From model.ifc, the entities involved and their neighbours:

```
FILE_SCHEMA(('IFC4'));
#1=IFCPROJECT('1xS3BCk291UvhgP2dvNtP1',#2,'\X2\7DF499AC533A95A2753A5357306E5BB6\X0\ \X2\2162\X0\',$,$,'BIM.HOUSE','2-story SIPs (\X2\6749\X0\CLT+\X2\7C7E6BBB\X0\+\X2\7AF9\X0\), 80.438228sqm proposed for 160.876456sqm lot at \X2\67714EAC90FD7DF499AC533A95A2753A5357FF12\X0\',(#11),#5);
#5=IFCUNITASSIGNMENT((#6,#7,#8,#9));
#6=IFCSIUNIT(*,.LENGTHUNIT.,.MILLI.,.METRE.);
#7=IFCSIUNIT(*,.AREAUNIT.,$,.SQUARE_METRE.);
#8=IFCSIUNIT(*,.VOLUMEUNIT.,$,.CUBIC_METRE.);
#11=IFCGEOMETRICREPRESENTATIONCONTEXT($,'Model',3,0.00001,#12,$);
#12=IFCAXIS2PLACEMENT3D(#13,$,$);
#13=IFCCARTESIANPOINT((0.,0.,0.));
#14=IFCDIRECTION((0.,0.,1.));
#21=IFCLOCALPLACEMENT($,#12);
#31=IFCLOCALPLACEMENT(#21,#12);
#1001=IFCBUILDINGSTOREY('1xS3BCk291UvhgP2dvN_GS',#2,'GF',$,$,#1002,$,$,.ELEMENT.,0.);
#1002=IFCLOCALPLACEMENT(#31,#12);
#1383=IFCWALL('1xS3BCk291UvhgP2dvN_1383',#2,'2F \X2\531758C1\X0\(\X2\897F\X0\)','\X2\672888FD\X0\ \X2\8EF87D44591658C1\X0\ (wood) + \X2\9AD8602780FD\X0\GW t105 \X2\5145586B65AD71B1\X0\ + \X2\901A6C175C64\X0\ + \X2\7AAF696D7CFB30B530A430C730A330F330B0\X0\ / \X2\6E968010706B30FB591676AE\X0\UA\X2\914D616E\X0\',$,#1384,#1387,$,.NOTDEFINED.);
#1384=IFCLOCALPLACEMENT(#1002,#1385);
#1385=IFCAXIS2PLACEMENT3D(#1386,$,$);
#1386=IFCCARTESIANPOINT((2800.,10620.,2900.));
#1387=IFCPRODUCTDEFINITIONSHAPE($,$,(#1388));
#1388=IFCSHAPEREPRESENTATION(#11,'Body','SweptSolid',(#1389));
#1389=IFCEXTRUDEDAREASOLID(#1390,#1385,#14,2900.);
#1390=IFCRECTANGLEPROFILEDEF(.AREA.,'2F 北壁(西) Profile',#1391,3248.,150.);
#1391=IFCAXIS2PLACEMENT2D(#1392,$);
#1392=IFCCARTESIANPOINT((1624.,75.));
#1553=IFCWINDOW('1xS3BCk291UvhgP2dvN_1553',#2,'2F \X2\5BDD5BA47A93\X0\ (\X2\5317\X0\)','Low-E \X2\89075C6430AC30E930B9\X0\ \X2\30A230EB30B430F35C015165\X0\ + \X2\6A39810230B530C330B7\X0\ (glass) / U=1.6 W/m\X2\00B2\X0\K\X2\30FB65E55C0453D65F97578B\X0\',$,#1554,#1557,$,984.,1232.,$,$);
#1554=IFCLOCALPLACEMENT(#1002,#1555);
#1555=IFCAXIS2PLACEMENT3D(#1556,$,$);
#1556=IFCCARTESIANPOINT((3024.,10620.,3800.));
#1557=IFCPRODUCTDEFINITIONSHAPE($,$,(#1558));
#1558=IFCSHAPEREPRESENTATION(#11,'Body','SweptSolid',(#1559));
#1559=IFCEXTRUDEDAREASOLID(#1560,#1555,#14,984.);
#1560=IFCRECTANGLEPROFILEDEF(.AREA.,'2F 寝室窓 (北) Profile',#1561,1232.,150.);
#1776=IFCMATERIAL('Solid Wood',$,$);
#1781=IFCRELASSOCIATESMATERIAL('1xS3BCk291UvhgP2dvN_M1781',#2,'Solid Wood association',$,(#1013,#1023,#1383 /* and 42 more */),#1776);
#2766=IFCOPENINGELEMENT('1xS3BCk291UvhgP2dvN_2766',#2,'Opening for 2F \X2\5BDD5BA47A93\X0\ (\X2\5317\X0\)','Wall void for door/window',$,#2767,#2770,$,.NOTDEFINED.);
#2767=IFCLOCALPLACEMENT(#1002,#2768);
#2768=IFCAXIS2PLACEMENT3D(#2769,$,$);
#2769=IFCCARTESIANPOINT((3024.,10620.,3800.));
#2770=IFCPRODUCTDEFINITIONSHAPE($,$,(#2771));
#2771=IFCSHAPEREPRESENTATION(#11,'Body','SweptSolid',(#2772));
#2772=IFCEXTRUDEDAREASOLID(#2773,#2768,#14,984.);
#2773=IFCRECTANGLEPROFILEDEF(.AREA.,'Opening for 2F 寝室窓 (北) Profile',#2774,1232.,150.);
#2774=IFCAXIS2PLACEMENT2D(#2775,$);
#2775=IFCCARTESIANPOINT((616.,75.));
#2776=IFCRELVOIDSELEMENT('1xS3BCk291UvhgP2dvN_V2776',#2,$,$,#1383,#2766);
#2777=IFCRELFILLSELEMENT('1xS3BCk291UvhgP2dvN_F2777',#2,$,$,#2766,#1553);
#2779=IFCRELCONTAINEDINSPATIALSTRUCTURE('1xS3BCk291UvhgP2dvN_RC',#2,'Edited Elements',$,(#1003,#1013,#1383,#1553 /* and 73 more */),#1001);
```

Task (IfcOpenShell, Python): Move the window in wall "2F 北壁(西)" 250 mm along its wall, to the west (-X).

```python
import ifcopenshell
import ifcopenshell.api.geometry
import ifcopenshell.util.placement

model = ifcopenshell.open("model.ifc")

window = model.by_guid("1xS3BCk291UvhgP2dvN_1553")
opening = window.FillsVoids[0].RelatingOpeningElement
wall = opening.VoidsElements[0].RelatingBuildingElement

wall_matrix = ifcopenshell.util.placement.get_local_placement(wall.ObjectPlacement)
shift = wall_matrix[:3, 0] * -250.0
before = ifcopenshell.util.placement.get_local_placement(window.ObjectPlacement)[:3, 3].copy()

# The window is not placed relative to its opening, so move both.
for product in (opening, window):
    matrix = ifcopenshell.util.placement.get_local_placement(product.ObjectPlacement)
    matrix[:3, 3] += shift
    ifcopenshell.api.geometry.edit_object_placement(model, product=product, matrix=matrix, is_si=False)

after = ifcopenshell.util.placement.get_local_placement(window.ObjectPlacement)[:3, 3]
print("window moved by", (after - before).round(3) + 0.0)

model.write("model_updated.ifc")
```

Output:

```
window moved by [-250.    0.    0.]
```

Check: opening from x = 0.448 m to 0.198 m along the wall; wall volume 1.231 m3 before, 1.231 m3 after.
